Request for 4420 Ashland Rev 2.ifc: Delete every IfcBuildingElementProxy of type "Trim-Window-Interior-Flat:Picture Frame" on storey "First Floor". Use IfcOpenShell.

First a look at what the model holds.

```python
import ifcopenshell
import ifcopenshell.util.element

model = ifcopenshell.open("4420 Ashland Rev 2.ifc")
print(model.schema)
storey = next(s for s in model.by_type("IfcBuildingStorey") if s.Name == "First Floor")
proxies = [e for e in ifcopenshell.util.element.get_decomposition(storey) if e.is_a("IfcBuildingElementProxy")]
seen = {}
for e in proxies:
    element_type = ifcopenshell.util.element.get_type(e)
    name = element_type.Name if element_type not in (None, e) else None
    seen[name] = seen.get(name, 0) + 1
for name, count in sorted(seen.items(), key=str):
    print(count, "x", name)
```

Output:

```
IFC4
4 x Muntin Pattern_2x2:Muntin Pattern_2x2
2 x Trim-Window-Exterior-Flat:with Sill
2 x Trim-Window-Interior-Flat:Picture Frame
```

```python
import ifcopenshell
import ifcopenshell.api.root
import ifcopenshell.util.element

model = ifcopenshell.open("4420 Ashland Rev 2.ifc")

storey = next(s for s in model.by_type("IfcBuildingStorey") if s.Name == "First Floor")
proxies = [e for e in ifcopenshell.util.element.get_decomposition(storey) if e.is_a("IfcBuildingElementProxy")]
targets = [e for e in proxies if (t := ifcopenshell.util.element.get_type(e)) not in (None, e) and t.Name == "Trim-Window-Interior-Flat:Picture Frame"]

for e in targets:
    ifcopenshell.api.root.remove_product(model, product=e)
print(len(targets), "removed")

model.write("4420 Ashland Rev 2_edited.ifc")
```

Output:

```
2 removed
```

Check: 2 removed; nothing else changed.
